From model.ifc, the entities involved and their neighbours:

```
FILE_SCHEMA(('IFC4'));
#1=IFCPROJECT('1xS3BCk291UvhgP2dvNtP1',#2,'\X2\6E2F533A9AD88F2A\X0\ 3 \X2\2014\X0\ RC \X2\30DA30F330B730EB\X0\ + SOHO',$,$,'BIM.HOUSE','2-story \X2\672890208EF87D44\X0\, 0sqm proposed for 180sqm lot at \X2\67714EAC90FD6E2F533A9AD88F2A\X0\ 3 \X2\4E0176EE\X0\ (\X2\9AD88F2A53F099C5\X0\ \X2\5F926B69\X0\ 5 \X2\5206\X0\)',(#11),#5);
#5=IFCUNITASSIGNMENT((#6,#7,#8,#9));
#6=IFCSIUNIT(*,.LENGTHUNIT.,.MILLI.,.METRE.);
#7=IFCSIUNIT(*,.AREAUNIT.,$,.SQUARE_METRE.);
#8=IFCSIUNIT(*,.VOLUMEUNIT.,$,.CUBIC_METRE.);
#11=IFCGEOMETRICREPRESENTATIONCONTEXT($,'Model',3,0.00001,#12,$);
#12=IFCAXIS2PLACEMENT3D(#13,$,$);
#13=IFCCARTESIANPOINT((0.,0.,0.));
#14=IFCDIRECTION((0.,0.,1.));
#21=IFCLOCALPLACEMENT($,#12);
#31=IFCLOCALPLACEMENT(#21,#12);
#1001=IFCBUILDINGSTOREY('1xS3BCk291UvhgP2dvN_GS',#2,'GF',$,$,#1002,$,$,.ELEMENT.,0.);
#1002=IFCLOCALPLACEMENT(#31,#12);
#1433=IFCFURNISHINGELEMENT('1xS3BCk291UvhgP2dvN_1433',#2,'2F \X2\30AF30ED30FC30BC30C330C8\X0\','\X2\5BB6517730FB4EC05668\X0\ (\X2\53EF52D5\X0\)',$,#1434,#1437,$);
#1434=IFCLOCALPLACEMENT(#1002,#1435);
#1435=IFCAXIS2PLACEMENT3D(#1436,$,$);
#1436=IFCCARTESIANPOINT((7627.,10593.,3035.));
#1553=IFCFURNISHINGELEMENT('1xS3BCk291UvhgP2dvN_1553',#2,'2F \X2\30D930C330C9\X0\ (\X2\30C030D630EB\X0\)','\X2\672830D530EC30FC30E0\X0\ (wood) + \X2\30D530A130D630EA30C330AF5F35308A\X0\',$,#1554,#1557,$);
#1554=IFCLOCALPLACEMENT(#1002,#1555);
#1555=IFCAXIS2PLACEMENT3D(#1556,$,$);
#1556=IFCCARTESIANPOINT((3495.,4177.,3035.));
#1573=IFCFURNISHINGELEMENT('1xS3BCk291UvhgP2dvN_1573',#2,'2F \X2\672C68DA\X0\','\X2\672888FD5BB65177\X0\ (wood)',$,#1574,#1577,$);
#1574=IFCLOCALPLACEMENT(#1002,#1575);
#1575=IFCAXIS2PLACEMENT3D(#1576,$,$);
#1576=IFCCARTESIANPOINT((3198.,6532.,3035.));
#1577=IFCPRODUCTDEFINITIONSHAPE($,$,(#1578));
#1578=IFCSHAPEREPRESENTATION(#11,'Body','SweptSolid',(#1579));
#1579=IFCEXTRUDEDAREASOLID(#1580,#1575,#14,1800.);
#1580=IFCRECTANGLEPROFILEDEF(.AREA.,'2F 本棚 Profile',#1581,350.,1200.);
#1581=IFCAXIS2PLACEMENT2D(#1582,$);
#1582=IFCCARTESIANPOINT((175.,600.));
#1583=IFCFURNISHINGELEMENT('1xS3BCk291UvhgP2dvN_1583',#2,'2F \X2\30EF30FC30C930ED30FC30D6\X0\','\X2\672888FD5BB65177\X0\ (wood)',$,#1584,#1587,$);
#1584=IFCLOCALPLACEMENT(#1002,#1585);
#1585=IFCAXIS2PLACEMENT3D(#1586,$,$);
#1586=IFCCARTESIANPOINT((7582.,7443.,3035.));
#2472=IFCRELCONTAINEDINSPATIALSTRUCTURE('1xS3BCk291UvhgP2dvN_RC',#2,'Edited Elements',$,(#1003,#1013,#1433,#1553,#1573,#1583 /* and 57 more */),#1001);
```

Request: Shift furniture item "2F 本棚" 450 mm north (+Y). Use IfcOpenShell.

```python
import ifcopenshell
import ifcopenshell.api.geometry
import ifcopenshell.util.placement

model = ifcopenshell.open("model.ifc")

item = model.by_id(1573)
matrix = ifcopenshell.util.placement.get_local_placement(item.ObjectPlacement)
matrix[1, 3] += 450.0
ifcopenshell.api.geometry.edit_object_placement(model, product=item, matrix=matrix, is_si=False)

print(ifcopenshell.util.placement.get_local_placement(item.ObjectPlacement).round(3) + 0.0)

model.write("model_rev.ifc")
```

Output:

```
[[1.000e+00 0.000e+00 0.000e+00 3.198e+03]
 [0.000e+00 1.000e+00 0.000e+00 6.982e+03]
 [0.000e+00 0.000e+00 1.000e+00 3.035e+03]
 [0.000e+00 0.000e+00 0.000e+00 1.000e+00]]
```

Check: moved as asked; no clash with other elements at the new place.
